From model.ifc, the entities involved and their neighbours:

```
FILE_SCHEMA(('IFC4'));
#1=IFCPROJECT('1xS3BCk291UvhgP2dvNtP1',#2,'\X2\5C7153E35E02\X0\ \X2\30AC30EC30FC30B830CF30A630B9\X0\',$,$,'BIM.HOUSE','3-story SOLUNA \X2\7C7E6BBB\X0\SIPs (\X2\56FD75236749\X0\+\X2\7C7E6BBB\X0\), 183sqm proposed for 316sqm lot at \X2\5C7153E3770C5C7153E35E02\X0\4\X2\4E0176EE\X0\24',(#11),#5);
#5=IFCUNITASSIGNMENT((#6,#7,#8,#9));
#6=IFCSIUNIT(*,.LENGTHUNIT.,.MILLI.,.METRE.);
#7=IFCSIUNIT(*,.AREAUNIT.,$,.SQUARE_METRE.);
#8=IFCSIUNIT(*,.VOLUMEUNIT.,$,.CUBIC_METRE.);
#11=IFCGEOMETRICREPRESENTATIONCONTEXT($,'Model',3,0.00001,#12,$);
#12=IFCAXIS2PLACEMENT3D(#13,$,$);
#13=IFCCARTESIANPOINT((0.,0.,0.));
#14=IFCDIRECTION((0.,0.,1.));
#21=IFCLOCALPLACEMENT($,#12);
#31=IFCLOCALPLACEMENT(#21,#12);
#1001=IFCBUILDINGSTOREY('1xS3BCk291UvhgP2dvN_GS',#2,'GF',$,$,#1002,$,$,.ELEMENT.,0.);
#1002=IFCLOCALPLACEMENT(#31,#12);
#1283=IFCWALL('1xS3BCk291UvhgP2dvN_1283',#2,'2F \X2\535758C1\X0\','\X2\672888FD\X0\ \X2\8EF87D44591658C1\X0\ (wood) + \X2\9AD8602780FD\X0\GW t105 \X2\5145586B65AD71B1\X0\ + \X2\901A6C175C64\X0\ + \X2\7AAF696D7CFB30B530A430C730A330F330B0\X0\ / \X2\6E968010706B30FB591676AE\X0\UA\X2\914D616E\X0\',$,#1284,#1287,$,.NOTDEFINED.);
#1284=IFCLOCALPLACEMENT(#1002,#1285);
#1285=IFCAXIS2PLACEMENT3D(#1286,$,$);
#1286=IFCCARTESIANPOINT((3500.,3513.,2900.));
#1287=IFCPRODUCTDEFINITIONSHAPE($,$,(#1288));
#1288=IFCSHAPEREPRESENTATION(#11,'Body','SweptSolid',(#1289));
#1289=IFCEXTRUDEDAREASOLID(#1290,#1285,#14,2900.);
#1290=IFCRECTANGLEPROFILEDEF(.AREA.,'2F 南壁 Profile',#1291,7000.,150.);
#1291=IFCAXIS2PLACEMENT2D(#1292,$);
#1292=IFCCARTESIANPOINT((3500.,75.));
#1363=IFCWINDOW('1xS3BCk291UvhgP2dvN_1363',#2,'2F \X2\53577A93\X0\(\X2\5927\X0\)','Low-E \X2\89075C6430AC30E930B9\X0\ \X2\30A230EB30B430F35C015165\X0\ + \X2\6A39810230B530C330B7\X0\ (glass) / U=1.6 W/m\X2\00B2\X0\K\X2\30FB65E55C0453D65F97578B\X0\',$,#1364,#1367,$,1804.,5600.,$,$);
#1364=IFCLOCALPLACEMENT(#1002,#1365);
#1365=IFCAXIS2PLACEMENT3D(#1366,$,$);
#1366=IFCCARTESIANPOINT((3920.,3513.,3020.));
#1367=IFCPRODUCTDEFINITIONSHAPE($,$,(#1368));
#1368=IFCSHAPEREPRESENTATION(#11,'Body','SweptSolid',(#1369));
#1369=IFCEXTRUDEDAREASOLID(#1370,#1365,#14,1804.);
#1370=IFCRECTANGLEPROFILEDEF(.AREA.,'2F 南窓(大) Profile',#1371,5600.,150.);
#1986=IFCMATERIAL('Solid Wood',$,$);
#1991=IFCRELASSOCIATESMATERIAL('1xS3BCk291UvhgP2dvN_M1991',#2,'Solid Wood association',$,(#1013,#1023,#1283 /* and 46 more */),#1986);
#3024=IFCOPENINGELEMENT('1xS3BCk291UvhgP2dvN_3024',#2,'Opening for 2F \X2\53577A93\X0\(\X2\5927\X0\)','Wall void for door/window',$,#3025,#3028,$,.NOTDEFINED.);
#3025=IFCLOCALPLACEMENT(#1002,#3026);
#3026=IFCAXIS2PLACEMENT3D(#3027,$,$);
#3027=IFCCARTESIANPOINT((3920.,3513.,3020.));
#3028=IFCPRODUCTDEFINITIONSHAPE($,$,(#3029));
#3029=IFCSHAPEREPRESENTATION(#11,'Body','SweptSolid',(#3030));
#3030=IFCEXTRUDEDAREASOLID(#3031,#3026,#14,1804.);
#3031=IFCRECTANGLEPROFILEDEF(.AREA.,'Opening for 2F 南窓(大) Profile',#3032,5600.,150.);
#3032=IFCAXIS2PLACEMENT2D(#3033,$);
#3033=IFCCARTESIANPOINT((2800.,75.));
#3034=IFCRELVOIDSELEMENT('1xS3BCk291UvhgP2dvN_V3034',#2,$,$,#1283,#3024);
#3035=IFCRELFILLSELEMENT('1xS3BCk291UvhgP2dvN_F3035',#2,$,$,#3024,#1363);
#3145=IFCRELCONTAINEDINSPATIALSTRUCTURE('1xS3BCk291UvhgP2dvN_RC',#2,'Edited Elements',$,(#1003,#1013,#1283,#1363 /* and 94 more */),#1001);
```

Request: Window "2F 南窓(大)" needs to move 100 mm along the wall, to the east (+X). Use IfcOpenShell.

```python
import ifcopenshell
import ifcopenshell.api.geometry
import ifcopenshell.util.placement
import ifcopenshell.util.unit

model = ifcopenshell.open("model.ifc")
unit_scale = ifcopenshell.util.unit.calculate_unit_scale(model)

window = model.by_guid("1xS3BCk291UvhgP2dvN_1363")
opening = window.FillsVoids[0].RelatingOpeningElement
wall = opening.VoidsElements[0].RelatingBuildingElement

wall_matrix = ifcopenshell.util.placement.get_local_placement(wall.ObjectPlacement)
shift = wall_matrix[:3, 0] * 0.1 / unit_scale
before = ifcopenshell.util.placement.get_local_placement(window.ObjectPlacement)[:3, 3].copy()

# The window is not placed relative to its opening, so move both.
for product in (opening, window):
    matrix = ifcopenshell.util.placement.get_local_placement(product.ObjectPlacement)
    matrix[:3, 3] += shift
    ifcopenshell.api.geometry.edit_object_placement(model, product=product, matrix=matrix, is_si=False)

after = ifcopenshell.util.placement.get_local_placement(window.ObjectPlacement)[:3, 3]
print("window moved by", (after - before).round(3) + 0.0)

model.write("model_v2.ifc")
```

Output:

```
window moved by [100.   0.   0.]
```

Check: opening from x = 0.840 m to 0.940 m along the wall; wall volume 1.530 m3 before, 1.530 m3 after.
